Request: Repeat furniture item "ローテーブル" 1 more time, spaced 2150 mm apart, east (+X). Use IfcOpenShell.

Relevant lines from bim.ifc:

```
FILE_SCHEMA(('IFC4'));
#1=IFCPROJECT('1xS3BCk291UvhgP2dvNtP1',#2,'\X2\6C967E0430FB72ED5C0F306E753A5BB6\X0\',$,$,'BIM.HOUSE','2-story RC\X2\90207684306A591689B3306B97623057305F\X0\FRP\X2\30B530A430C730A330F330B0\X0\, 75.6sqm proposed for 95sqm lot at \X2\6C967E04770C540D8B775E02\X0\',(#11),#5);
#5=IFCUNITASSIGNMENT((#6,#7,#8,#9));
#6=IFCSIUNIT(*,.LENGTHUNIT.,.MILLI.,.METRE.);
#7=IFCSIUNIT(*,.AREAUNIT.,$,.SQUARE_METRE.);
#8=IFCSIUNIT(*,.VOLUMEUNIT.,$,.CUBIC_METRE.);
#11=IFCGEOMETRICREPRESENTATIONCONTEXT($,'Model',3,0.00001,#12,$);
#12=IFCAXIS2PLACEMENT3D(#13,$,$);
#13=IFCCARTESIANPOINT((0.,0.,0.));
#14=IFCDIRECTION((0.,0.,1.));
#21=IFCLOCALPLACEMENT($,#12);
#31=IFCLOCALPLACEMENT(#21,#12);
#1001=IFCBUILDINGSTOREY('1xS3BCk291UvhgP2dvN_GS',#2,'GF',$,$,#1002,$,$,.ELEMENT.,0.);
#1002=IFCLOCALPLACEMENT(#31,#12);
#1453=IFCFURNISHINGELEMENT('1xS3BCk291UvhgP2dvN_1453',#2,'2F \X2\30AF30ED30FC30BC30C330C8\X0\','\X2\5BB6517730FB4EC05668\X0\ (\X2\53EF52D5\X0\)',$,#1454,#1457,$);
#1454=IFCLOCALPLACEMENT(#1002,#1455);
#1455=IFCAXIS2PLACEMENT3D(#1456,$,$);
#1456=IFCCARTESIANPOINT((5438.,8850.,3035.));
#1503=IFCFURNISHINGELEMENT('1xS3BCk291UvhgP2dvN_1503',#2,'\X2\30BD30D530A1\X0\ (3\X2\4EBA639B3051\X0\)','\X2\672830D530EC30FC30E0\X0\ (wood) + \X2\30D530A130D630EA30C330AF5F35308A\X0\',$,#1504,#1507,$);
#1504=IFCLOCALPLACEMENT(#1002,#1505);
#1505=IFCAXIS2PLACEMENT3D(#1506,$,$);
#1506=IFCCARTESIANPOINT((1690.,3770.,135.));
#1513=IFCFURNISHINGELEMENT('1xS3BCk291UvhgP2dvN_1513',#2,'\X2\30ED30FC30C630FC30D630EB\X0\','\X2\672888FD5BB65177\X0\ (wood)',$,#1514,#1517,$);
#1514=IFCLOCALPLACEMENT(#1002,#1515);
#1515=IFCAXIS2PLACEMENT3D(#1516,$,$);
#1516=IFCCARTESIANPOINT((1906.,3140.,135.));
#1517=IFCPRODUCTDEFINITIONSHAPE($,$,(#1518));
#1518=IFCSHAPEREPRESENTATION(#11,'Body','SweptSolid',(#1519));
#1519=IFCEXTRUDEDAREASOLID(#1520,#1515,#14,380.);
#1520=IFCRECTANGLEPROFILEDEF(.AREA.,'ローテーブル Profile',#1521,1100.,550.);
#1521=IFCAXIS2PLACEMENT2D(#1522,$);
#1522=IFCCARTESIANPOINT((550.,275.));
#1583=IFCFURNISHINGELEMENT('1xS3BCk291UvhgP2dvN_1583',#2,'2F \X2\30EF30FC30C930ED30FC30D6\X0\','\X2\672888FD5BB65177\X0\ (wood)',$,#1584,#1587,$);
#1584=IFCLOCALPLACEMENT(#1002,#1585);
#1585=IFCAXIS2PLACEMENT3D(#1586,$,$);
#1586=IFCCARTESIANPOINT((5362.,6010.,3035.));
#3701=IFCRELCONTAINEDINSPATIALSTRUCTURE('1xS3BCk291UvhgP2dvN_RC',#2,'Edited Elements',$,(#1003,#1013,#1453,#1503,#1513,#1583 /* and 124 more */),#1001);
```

```python
import numpy as np
import ifcopenshell
import ifcopenshell.api.geometry
import ifcopenshell.api.root
import ifcopenshell.util.element
import ifcopenshell.util.placement
import ifcopenshell.util.unit

model = ifcopenshell.open("bim.ifc")
unit_scale = ifcopenshell.util.unit.calculate_unit_scale(model)


def reuse_history(source, copy):
    """copy_class also copies each property set's owner history, people and application; keep the originals."""
    for rel in copy.IsDefinedBy:
        if rel.is_a("IfcRelDefinesByProperties") and (history := rel.RelatingPropertyDefinition.OwnerHistory):
            rel.RelatingPropertyDefinition.OwnerHistory = source.OwnerHistory
            ifcopenshell.util.element.remove_deep2(model, history)


source = model.by_guid("1xS3BCk291UvhgP2dvN_1513")
base = ifcopenshell.util.placement.get_local_placement(source.ObjectPlacement)
step = np.array([1.0, 0.0, 0.0]) * 2.15 / unit_scale

for i in range(1, 2):
    copy = ifcopenshell.api.root.copy_class(model, product=source)
    copy.Representation = ifcopenshell.util.element.copy_deep(
        model, source.Representation, exclude=["IfcGeometricRepresentationContext", "IfcRepresentationMap"]
    )
    reuse_history(source, copy)
    matrix = base.copy()
    matrix[:3, 3] += i * step
    print("added at", matrix[:3, 3].round(3) + 0.0)
    ifcopenshell.api.geometry.edit_object_placement(model, product=copy, matrix=matrix, is_si=False)

model.write("bim_updated.ifc")
```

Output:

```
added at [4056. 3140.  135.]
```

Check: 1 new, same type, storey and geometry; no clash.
